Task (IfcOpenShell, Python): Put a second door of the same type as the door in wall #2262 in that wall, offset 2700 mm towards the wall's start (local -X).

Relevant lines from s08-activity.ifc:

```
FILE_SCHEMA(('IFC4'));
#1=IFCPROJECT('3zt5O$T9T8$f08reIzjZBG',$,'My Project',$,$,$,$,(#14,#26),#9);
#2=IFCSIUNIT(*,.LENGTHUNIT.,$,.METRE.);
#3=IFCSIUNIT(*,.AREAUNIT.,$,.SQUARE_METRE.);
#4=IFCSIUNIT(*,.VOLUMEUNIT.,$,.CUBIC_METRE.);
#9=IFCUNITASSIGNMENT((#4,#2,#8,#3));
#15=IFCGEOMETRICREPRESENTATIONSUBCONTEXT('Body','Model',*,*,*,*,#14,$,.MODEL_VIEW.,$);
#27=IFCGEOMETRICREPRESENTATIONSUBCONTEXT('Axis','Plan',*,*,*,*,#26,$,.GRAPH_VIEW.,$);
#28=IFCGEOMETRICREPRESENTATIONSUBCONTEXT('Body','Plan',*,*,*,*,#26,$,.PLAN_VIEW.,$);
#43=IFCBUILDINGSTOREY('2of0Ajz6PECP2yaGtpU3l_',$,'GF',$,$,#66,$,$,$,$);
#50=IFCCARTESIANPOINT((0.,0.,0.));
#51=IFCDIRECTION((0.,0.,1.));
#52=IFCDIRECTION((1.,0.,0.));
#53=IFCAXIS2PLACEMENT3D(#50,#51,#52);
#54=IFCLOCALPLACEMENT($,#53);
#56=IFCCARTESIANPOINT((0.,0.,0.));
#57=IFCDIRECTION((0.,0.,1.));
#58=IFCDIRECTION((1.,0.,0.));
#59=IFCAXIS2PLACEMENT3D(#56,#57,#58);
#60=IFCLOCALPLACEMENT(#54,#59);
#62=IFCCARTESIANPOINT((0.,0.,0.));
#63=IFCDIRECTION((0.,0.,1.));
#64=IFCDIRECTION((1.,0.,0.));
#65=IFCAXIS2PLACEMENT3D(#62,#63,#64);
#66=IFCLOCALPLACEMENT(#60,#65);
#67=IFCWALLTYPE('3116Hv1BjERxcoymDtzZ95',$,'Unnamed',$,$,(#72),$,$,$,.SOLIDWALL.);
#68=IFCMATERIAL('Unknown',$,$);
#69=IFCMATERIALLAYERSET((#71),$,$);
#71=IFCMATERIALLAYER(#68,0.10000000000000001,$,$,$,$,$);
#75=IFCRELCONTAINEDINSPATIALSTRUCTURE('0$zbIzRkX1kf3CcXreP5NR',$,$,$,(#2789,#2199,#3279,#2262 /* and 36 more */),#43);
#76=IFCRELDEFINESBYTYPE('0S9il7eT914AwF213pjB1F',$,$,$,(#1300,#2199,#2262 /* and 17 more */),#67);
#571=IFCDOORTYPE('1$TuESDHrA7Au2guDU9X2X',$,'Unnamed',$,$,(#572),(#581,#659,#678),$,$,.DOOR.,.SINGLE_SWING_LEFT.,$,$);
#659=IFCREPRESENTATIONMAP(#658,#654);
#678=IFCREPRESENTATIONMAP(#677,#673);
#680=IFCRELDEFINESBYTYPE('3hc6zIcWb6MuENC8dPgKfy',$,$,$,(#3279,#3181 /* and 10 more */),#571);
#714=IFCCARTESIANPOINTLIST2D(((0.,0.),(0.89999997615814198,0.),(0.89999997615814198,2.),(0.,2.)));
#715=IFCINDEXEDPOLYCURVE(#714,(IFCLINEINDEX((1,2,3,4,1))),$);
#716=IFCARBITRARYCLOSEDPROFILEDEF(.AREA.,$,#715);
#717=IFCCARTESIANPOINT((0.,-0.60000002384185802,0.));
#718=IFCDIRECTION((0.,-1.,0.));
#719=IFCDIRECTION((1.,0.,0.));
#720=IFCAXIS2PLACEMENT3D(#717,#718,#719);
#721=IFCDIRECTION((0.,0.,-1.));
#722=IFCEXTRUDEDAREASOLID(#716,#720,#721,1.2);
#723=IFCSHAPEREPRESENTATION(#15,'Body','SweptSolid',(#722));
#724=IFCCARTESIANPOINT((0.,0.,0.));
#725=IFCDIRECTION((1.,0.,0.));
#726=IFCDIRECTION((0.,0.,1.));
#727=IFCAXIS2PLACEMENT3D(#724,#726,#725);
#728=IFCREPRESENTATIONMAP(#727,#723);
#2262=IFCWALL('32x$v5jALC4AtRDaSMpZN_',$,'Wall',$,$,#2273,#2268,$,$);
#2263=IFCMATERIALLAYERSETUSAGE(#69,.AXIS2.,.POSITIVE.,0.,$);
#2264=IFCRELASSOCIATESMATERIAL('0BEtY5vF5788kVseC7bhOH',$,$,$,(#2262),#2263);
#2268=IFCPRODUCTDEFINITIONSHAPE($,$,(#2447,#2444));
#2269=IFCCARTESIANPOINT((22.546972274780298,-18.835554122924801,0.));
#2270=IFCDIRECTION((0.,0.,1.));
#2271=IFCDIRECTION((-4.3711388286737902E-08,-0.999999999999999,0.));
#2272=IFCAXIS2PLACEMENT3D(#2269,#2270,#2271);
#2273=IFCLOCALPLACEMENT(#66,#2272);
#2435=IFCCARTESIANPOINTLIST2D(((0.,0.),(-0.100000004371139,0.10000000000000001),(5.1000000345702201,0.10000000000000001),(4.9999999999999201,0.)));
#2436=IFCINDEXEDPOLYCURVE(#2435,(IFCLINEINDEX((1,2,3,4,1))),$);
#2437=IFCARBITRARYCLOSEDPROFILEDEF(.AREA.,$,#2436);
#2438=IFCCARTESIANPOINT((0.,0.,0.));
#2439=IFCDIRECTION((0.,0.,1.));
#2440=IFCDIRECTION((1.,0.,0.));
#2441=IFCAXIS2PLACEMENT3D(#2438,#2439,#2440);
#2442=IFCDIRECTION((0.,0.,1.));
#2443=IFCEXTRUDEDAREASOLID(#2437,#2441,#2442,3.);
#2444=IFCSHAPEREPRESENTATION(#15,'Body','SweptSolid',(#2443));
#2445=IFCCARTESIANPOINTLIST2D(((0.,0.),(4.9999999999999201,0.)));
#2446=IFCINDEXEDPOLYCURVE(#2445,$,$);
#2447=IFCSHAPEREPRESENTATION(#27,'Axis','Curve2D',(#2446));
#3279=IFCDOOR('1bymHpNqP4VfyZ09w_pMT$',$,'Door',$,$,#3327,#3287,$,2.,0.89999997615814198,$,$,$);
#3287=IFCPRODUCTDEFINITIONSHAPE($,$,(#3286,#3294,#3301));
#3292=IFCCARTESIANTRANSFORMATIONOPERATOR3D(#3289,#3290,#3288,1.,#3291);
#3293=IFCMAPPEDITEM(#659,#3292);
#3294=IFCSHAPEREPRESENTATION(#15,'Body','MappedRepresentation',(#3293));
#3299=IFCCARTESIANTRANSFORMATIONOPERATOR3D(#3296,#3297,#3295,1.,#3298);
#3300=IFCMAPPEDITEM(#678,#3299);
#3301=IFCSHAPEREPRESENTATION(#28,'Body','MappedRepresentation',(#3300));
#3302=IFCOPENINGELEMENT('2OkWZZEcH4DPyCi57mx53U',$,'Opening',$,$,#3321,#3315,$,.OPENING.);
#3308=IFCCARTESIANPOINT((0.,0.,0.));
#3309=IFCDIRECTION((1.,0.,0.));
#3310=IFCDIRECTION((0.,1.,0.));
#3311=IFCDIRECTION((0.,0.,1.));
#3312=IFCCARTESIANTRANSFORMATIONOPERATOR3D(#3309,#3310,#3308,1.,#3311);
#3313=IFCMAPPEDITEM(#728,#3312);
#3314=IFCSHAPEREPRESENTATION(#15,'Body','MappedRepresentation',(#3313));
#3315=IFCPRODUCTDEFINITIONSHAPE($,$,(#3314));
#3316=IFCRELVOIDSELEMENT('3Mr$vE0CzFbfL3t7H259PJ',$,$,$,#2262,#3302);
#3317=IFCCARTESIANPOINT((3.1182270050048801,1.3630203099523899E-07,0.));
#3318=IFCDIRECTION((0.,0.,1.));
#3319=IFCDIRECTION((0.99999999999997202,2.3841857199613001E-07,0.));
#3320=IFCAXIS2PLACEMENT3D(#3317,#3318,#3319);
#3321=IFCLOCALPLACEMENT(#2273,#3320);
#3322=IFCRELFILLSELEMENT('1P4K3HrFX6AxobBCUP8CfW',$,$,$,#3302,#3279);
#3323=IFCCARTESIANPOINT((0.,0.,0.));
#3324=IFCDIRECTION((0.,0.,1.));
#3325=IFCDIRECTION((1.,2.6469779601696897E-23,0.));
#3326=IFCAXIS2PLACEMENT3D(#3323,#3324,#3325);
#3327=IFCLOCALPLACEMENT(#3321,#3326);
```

```python
import ifcopenshell
import ifcopenshell.api.feature
import ifcopenshell.api.geometry
import ifcopenshell.api.root
import ifcopenshell.geom
import ifcopenshell.util.element
import ifcopenshell.util.placement
import ifcopenshell.util.shape
import ifcopenshell.util.unit

model = ifcopenshell.open("s08-activity.ifc")
unit_scale = ifcopenshell.util.unit.calculate_unit_scale(model)
settings = ifcopenshell.geom.settings()


def volume(element):
    """Net volume in cubic metres, openings subtracted."""
    shape = ifcopenshell.geom.create_shape(settings, element)
    return ifcopenshell.util.shape.get_volume(shape.geometry)


door = model.by_guid("1bymHpNqP4VfyZ09w_pMT$")
opening = door.FillsVoids[0].RelatingOpeningElement
wall = opening.VoidsElements[0].RelatingBuildingElement
before = volume(wall)
shift = ifcopenshell.util.placement.get_local_placement(wall.ObjectPlacement)[:3, 0] * -2.7 / unit_scale

# copy_class copies the void relationship, type, container and properties, but no geometry.
new_opening = ifcopenshell.api.root.copy_class(model, product=opening)
new_opening.Representation = ifcopenshell.util.element.copy_deep(
    model, opening.Representation, exclude=["IfcGeometricRepresentationContext", "IfcRepresentationMap"]
)
new_door = ifcopenshell.api.root.copy_class(model, product=door)
new_door.Representation = ifcopenshell.util.element.copy_deep(
    model, door.Representation, exclude=["IfcGeometricRepresentationContext", "IfcRepresentationMap"]
)
ifcopenshell.api.feature.add_filling(model, opening=new_opening, element=new_door)

for old, new in ((opening, new_opening), (door, new_door)):
    matrix = ifcopenshell.util.placement.get_local_placement(old.ObjectPlacement)
    matrix[:3, 3] += shift
    ifcopenshell.api.geometry.edit_object_placement(model, product=new, matrix=matrix, is_si=False)

after = volume(wall)

print(f"wall volume {before:.3f} -> {after:.3f} m3")

model.write("s08-activity-out.ifc")
```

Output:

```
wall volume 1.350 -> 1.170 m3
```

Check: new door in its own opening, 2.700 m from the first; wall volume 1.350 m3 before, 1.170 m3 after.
